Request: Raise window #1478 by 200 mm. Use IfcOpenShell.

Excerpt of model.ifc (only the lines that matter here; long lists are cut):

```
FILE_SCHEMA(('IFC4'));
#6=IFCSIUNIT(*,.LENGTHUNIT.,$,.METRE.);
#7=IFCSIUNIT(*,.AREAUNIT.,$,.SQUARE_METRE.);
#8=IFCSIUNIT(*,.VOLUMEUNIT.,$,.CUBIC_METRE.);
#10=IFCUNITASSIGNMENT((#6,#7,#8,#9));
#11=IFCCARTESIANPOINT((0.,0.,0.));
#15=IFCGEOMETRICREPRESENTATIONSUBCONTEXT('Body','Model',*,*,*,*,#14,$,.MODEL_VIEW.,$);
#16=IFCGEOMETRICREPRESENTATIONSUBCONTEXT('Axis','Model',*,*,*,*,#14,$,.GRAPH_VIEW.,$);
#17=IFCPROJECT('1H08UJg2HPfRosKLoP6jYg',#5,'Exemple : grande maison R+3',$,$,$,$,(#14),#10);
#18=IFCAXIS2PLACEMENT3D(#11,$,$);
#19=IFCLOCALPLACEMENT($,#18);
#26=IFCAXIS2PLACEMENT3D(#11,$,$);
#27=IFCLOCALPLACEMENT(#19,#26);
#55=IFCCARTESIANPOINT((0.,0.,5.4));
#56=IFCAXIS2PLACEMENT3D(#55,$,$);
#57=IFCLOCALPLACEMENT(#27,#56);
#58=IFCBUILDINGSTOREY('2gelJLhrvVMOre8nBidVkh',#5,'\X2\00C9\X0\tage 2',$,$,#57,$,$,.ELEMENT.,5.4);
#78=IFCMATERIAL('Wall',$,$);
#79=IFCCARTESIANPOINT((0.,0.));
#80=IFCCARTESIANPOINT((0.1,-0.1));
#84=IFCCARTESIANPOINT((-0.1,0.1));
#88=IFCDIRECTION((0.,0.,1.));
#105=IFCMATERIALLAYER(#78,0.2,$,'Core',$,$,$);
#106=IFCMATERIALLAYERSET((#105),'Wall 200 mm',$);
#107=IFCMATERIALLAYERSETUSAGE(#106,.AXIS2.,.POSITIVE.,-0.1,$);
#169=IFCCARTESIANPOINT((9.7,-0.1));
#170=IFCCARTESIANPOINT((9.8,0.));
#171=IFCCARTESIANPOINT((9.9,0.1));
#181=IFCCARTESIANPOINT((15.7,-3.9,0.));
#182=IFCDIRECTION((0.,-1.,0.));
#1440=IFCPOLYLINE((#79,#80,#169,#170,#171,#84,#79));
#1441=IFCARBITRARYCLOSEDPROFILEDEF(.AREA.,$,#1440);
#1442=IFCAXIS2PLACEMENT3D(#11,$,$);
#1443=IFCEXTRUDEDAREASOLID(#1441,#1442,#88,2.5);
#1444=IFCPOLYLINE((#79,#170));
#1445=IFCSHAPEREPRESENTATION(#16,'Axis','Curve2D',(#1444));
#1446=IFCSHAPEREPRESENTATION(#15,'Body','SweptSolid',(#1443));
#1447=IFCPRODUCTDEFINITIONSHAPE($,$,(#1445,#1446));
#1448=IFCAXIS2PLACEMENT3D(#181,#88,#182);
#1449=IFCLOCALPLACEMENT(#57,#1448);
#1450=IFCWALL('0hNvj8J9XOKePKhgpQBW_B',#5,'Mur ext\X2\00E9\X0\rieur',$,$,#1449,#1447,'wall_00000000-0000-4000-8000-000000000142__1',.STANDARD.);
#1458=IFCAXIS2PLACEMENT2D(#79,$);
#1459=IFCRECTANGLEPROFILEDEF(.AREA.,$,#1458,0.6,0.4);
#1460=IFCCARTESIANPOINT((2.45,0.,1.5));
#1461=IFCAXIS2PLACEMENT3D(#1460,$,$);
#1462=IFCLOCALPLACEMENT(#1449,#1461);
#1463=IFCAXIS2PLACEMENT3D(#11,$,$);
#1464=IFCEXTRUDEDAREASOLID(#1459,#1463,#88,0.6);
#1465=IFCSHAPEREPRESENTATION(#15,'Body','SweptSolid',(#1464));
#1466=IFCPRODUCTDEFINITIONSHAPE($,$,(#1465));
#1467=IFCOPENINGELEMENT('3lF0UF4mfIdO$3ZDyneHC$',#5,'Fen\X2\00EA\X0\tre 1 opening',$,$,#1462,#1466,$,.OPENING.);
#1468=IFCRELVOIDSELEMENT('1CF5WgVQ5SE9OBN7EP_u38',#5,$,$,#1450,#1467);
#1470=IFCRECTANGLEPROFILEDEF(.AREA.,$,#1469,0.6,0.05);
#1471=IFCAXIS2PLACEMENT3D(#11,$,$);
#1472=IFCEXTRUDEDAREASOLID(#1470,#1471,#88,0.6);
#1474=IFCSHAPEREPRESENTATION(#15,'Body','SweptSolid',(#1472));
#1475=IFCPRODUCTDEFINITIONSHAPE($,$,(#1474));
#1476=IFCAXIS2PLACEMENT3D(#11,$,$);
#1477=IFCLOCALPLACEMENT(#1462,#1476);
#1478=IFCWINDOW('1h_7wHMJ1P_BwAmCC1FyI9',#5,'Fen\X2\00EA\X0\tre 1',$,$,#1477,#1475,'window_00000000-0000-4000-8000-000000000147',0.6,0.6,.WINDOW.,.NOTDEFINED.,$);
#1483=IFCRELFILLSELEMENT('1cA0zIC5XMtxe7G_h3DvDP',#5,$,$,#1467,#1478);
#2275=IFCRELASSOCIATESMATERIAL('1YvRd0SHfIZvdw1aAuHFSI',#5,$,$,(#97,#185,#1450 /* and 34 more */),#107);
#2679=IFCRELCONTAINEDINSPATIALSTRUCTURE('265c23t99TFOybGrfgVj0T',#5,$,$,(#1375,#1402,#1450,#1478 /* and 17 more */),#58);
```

```python
import numpy as np
import ifcopenshell
import ifcopenshell.api.geometry
import ifcopenshell.util.placement
import ifcopenshell.util.unit

model = ifcopenshell.open("model.ifc")
unit_scale = ifcopenshell.util.unit.calculate_unit_scale(model)

window = model.by_id(1478)
opening = window.FillsVoids[0].RelatingOpeningElement
dz = 0.2 / unit_scale

shift = np.array([0.0, 0.0, dz])
# The window is placed relative to its opening, so it follows when the opening moves.
matrix = ifcopenshell.util.placement.get_local_placement(opening.ObjectPlacement)
matrix[:3, 3] += shift
ifcopenshell.api.geometry.edit_object_placement(
    model, product=opening, matrix=matrix, is_si=False, should_transform_children=True
)

print(f"moved by {dz * unit_scale:+.3f} m")

model.write("model_v2.ifc")
```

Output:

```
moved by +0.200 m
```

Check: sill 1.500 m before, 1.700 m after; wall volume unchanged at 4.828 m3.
